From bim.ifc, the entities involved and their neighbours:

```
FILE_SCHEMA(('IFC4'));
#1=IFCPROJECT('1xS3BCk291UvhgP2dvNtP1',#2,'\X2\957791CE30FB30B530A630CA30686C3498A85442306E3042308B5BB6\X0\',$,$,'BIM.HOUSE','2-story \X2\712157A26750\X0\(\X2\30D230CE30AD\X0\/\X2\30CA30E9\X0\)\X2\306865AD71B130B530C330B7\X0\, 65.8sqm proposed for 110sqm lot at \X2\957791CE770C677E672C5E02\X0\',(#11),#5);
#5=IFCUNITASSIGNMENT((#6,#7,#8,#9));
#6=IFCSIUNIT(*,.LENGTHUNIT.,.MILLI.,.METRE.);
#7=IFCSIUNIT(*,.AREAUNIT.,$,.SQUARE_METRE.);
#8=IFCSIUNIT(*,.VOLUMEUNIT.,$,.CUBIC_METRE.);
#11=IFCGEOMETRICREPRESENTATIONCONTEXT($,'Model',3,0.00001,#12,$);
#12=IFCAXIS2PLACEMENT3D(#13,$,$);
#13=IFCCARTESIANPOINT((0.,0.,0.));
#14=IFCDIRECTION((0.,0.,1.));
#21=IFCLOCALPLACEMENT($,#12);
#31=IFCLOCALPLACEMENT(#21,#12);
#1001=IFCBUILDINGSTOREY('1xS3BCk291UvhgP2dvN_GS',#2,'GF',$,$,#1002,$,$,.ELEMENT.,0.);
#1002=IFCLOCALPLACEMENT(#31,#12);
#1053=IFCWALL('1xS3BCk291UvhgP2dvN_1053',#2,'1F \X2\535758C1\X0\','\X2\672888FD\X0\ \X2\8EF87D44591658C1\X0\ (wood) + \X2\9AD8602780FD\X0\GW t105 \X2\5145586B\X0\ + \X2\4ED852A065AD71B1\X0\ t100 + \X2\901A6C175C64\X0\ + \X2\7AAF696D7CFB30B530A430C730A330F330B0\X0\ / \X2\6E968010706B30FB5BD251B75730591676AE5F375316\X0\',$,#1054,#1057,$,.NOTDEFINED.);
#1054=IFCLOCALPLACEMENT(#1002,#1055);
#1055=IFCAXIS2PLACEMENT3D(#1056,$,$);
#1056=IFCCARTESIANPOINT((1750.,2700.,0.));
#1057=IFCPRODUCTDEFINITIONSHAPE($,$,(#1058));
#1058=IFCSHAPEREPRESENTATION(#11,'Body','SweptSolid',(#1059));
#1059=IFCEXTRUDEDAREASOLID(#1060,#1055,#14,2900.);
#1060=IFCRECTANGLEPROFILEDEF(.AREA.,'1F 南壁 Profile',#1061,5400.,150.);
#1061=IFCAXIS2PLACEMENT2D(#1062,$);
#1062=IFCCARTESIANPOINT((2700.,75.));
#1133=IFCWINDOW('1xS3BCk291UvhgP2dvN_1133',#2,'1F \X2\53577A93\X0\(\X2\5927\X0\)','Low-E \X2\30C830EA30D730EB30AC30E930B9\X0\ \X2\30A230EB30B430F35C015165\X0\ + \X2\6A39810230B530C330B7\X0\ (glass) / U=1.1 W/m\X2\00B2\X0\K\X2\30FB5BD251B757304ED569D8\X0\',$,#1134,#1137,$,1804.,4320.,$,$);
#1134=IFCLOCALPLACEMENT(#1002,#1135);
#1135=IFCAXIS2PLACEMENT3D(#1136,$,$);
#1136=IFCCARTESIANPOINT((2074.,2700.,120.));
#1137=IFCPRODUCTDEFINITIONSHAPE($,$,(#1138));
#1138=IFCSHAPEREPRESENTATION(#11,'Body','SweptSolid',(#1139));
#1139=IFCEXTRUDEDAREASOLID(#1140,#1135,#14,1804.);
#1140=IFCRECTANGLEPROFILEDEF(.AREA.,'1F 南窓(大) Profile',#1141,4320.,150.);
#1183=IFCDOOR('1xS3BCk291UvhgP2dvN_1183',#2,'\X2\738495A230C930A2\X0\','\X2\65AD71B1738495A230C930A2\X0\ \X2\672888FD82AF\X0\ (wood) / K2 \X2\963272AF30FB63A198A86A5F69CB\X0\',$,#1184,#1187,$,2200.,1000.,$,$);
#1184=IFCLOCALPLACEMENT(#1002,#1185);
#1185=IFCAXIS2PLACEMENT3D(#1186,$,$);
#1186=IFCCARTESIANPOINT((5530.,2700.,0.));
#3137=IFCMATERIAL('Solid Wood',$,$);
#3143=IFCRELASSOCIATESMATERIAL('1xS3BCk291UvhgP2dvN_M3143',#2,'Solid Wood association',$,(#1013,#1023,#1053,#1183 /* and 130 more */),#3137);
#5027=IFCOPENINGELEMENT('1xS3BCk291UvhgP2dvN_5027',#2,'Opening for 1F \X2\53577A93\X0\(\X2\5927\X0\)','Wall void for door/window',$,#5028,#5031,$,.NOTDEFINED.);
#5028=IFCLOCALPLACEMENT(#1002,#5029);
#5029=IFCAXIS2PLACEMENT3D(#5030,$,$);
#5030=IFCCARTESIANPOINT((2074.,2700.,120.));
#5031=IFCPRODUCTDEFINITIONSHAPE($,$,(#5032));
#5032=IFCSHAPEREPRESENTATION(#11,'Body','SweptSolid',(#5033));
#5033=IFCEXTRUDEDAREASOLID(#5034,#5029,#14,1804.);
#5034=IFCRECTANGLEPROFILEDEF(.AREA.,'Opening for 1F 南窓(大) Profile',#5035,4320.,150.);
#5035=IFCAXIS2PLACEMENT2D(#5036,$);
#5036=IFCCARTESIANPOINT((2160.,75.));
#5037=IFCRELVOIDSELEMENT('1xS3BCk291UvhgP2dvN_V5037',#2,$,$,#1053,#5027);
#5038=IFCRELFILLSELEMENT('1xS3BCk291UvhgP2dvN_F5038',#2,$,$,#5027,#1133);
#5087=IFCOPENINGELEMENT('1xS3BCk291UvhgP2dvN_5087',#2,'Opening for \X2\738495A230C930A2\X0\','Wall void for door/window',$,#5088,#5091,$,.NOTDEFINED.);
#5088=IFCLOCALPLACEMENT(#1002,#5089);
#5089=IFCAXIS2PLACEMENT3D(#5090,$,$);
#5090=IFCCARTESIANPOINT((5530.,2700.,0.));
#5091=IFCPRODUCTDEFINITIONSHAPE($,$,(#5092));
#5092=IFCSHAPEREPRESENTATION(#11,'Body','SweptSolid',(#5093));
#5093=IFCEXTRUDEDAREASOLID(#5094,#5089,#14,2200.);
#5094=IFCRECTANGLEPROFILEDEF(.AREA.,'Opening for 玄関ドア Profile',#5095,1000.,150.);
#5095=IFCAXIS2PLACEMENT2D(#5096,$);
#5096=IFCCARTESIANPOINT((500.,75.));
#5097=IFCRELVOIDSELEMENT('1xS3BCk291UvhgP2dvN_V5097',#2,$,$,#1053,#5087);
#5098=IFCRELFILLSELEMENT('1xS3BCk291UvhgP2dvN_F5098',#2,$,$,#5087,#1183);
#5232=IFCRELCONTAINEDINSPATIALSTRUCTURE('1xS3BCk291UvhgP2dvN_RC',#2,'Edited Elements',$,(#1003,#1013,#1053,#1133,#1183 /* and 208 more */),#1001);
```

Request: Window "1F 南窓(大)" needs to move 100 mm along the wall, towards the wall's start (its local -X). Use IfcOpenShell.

```python
import ifcopenshell
import ifcopenshell.api.geometry
import ifcopenshell.util.placement
import ifcopenshell.util.unit

model = ifcopenshell.open("bim.ifc")
unit_scale = ifcopenshell.util.unit.calculate_unit_scale(model)

window = model.by_id(1133)
opening = window.FillsVoids[0].RelatingOpeningElement
wall = opening.VoidsElements[0].RelatingBuildingElement

wall_matrix = ifcopenshell.util.placement.get_local_placement(wall.ObjectPlacement)
shift = wall_matrix[:3, 0] * -0.1 / unit_scale
before = ifcopenshell.util.placement.get_local_placement(window.ObjectPlacement)[:3, 3].copy()

# The window is not placed relative to its opening, so move both.
for product in (opening, window):
    matrix = ifcopenshell.util.placement.get_local_placement(product.ObjectPlacement)
    matrix[:3, 3] += shift
    ifcopenshell.api.geometry.edit_object_placement(model, product=product, matrix=matrix, is_si=False)

after = ifcopenshell.util.placement.get_local_placement(window.ObjectPlacement)[:3, 3]
print("window moved by", (after - before).round(3) + 0.0)

model.write("bim_rev.ifc")
```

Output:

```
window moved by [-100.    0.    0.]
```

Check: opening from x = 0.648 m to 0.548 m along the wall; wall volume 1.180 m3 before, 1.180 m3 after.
